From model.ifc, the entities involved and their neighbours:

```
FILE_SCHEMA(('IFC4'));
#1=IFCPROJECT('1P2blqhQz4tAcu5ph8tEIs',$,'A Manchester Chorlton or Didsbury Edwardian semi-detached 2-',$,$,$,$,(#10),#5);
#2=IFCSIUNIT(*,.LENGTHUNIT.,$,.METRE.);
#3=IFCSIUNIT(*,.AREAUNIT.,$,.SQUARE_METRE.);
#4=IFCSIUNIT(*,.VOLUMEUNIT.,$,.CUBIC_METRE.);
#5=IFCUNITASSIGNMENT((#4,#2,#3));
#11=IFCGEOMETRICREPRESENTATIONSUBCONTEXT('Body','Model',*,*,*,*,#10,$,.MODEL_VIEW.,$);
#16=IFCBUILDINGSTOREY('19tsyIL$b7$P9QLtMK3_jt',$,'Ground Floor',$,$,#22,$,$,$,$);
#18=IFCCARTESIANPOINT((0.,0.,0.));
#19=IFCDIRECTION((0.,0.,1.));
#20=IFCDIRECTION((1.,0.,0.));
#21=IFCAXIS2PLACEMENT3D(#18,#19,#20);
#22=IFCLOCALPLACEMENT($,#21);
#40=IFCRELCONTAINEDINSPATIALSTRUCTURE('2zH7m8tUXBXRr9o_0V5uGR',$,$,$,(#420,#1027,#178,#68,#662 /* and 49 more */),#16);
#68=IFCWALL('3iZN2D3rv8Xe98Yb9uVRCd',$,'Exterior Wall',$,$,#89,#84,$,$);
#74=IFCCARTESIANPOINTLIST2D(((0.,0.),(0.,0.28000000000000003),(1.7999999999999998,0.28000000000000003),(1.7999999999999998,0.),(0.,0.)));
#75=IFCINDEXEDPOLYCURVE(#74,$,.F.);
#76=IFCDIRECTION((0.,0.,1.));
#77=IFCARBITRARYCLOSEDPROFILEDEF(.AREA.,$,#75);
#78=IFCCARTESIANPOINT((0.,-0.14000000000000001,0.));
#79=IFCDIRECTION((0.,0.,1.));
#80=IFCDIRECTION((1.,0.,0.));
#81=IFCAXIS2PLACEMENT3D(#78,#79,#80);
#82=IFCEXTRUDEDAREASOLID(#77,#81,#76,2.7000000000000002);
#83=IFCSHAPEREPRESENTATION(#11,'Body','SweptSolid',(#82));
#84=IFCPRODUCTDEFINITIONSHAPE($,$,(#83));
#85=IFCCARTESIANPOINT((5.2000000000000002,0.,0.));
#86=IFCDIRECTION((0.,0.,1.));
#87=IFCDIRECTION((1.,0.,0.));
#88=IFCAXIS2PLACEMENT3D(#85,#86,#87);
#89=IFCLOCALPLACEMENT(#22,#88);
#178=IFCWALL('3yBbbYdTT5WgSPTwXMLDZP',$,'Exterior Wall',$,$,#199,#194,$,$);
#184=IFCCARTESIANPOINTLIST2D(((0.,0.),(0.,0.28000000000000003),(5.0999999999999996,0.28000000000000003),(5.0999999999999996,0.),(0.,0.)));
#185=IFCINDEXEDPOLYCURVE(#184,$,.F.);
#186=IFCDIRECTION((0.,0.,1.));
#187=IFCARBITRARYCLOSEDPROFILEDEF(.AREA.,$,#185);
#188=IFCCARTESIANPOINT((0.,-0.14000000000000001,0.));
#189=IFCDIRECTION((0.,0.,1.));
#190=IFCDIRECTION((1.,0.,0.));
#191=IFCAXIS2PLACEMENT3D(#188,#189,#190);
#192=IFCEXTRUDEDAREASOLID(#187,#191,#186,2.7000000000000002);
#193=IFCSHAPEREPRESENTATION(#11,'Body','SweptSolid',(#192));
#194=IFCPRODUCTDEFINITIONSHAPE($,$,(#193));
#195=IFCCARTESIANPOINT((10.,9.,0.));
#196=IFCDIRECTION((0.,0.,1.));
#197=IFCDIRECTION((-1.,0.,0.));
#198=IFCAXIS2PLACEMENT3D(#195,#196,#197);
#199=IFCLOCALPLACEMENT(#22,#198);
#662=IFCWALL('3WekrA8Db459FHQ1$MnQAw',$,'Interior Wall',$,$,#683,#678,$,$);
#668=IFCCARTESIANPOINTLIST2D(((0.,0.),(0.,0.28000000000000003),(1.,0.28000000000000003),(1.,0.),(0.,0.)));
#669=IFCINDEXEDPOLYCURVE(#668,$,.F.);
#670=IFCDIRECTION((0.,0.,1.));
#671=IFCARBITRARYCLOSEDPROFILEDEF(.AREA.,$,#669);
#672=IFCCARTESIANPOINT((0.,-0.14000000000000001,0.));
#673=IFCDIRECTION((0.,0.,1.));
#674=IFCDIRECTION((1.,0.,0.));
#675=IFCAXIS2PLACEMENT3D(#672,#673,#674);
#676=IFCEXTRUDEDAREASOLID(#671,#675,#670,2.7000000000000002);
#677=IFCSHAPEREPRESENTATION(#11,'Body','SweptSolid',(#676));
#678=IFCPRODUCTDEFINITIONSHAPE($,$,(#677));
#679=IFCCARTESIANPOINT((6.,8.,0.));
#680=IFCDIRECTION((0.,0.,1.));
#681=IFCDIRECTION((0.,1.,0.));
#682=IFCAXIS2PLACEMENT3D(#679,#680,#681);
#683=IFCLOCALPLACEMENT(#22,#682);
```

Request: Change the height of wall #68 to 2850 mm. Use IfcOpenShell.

```python
import ifcopenshell
import ifcopenshell.geom
import ifcopenshell.util.representation
import ifcopenshell.util.shape
import ifcopenshell.util.unit

model = ifcopenshell.open("model.ifc")
unit_scale = ifcopenshell.util.unit.calculate_unit_scale(model)
settings = ifcopenshell.geom.settings()


def volume(element):
    """Net volume in cubic metres, openings subtracted."""
    shape = ifcopenshell.geom.create_shape(settings, element)
    return ifcopenshell.util.shape.get_volume(shape.geometry)


wall = model.by_guid("3iZN2D3rv8Xe98Yb9uVRCd")
before = volume(wall)

body = ifcopenshell.util.representation.get_representation(wall, "Model", "Body")
solid = body.Items[0]
old_height = solid.Depth
solid.Depth = 2.85 / unit_scale
after = volume(wall)

print(f"height {old_height:g} -> {solid.Depth:g}, volume {before:.3f} -> {after:.3f} m3")

model.write("model_edited.ifc")
```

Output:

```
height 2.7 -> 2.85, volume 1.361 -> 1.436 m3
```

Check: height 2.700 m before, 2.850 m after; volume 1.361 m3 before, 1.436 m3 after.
